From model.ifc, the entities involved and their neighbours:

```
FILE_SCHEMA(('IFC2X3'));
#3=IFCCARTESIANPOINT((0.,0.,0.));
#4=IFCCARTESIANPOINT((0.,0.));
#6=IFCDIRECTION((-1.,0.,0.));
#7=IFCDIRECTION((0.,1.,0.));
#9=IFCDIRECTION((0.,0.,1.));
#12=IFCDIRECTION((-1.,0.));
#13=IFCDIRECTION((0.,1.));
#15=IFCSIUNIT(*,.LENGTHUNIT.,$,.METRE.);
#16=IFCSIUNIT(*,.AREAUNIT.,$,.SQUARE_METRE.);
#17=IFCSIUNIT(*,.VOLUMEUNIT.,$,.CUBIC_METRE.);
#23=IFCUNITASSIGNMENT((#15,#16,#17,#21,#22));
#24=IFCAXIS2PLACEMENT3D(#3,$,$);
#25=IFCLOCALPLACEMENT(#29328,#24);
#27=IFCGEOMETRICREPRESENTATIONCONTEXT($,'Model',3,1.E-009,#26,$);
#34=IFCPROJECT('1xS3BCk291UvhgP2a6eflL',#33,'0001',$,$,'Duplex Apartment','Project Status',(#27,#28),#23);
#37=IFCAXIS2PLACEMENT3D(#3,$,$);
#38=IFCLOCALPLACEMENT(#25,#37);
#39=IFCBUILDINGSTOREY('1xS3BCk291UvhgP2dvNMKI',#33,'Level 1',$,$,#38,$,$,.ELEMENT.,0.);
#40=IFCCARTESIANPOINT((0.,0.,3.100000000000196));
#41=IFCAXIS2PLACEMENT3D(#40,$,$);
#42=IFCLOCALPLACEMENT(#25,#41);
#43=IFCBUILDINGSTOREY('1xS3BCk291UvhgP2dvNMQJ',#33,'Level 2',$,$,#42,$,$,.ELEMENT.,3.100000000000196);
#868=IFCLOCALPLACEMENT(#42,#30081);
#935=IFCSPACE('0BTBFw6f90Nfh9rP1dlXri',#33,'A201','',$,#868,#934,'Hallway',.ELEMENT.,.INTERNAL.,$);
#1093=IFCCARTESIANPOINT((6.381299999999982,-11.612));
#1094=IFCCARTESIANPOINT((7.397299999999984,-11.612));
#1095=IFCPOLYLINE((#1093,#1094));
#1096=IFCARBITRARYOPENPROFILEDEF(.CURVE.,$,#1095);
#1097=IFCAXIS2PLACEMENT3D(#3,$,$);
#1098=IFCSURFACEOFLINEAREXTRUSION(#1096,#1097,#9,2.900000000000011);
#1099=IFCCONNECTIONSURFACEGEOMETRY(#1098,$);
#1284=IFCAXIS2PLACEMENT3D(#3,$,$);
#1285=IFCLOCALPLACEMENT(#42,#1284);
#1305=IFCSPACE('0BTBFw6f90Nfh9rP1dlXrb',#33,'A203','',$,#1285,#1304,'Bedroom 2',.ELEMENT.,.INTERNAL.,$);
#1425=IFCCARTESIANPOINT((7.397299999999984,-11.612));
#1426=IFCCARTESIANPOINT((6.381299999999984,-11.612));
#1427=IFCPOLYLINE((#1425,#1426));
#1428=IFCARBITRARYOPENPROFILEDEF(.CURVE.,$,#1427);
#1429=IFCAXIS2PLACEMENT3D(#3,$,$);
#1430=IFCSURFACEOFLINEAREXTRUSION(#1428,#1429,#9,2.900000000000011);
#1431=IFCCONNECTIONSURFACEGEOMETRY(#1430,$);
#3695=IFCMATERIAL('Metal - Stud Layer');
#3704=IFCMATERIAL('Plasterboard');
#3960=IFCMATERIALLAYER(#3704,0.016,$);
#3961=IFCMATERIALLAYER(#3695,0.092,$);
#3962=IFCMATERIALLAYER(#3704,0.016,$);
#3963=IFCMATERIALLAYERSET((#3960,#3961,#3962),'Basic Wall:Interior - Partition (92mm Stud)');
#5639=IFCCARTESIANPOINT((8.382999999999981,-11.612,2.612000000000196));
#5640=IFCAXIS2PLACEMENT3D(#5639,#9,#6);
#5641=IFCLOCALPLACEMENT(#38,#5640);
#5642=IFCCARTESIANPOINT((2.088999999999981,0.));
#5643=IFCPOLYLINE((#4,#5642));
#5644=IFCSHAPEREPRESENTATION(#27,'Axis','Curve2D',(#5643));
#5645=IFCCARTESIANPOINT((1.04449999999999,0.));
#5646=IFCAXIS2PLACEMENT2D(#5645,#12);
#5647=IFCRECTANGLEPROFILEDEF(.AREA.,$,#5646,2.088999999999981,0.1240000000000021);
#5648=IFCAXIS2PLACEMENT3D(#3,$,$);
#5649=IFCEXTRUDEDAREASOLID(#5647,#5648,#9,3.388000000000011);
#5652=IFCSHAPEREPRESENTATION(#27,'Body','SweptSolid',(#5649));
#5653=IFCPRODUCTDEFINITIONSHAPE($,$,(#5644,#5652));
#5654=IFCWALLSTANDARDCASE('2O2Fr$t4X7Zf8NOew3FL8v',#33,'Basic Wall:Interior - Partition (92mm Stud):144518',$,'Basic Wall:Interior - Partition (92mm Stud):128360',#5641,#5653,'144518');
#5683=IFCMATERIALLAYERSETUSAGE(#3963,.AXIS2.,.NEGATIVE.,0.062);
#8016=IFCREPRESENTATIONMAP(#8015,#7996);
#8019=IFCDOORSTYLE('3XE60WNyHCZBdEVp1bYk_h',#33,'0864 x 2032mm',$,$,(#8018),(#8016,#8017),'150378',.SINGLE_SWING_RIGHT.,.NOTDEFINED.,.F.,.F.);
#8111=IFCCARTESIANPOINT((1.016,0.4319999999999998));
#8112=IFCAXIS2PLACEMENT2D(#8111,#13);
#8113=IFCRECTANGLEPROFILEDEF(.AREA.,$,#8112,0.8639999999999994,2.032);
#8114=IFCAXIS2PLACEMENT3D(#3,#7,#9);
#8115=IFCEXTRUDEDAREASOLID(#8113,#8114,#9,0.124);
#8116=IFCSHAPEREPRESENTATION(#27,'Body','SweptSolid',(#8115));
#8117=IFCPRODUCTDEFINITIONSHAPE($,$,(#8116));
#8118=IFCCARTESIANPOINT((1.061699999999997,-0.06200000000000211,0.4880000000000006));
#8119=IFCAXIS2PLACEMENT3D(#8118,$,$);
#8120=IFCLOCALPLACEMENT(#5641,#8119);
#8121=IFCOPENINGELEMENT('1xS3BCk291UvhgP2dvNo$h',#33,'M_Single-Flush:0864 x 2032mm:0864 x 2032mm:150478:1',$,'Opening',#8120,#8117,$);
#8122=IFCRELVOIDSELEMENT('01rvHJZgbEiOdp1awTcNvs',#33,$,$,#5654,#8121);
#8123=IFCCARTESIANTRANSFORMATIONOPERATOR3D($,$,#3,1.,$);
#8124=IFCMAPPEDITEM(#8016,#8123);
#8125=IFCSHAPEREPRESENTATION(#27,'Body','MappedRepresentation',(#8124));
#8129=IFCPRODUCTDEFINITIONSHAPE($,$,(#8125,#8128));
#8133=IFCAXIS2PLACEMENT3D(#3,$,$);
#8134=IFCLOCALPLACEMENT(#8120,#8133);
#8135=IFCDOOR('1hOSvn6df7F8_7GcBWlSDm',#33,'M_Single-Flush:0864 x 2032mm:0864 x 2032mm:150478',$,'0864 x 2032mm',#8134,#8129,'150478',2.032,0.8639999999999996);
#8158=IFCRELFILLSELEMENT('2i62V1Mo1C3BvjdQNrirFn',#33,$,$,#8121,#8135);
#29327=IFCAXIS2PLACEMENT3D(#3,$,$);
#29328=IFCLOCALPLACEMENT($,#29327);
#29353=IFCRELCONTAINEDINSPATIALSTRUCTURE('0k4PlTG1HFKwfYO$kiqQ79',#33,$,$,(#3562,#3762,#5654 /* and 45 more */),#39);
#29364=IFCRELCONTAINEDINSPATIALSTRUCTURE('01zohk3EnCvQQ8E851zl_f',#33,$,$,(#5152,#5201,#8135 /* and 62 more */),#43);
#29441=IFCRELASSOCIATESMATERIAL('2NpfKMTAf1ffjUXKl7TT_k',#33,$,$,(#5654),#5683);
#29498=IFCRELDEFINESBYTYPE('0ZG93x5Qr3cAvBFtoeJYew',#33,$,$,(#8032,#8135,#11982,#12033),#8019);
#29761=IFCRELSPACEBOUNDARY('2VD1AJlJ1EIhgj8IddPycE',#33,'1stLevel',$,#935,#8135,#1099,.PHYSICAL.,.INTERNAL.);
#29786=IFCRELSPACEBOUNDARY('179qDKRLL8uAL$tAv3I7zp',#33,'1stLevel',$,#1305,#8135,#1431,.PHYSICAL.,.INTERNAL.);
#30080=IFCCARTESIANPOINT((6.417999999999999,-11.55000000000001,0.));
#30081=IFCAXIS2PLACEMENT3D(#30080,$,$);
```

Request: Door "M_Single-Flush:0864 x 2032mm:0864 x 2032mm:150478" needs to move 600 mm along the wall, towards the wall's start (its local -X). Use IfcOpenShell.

```python
import numpy as np
import ifcopenshell
import ifcopenshell.api.geometry
import ifcopenshell.util.placement
import ifcopenshell.util.unit

model = ifcopenshell.open("model.ifc")
unit_scale = ifcopenshell.util.unit.calculate_unit_scale(model)

door = model.by_guid("1hOSvn6df7F8_7GcBWlSDm")
opening = door.FillsVoids[0].RelatingOpeningElement
wall = opening.VoidsElements[0].RelatingBuildingElement

wall_matrix = ifcopenshell.util.placement.get_local_placement(wall.ObjectPlacement)
shift = wall_matrix[:3, 0] * -0.6 / unit_scale
before = ifcopenshell.util.placement.get_local_placement(door.ObjectPlacement)[:3, 3].copy()

# The door is placed relative to its opening, so it follows when the opening moves.
matrix = ifcopenshell.util.placement.get_local_placement(opening.ObjectPlacement)
matrix[:3, 3] += shift
ifcopenshell.api.geometry.edit_object_placement(
    model, product=opening, matrix=matrix, is_si=False, should_transform_children=True
)

# Space boundary surfaces are stored in each space's coordinates; move them too.
for rel in door.ProvidesBoundaries:
    if not rel.ConnectionGeometry:
        continue
    surface = rel.ConnectionGeometry.SurfaceOnRelatingElement
    space_matrix = ifcopenshell.util.placement.get_local_placement(rel.RelatingSpace.ObjectPlacement)
    point = np.array(surface.Position.Location.Coordinates) + space_matrix[:3, :3].T @ shift
    surface.Position = model.createIfcAxis2Placement3D(
        model.createIfcCartesianPoint(point.tolist()), surface.Position.Axis, surface.Position.RefDirection
    )

after = ifcopenshell.util.placement.get_local_placement(door.ObjectPlacement)[:3, 3]
print("door moved by", (after - before).round(3) + 0.0)

model.write("model_rev.ifc")
```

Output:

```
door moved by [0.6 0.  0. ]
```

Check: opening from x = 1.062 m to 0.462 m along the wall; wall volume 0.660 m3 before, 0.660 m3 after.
